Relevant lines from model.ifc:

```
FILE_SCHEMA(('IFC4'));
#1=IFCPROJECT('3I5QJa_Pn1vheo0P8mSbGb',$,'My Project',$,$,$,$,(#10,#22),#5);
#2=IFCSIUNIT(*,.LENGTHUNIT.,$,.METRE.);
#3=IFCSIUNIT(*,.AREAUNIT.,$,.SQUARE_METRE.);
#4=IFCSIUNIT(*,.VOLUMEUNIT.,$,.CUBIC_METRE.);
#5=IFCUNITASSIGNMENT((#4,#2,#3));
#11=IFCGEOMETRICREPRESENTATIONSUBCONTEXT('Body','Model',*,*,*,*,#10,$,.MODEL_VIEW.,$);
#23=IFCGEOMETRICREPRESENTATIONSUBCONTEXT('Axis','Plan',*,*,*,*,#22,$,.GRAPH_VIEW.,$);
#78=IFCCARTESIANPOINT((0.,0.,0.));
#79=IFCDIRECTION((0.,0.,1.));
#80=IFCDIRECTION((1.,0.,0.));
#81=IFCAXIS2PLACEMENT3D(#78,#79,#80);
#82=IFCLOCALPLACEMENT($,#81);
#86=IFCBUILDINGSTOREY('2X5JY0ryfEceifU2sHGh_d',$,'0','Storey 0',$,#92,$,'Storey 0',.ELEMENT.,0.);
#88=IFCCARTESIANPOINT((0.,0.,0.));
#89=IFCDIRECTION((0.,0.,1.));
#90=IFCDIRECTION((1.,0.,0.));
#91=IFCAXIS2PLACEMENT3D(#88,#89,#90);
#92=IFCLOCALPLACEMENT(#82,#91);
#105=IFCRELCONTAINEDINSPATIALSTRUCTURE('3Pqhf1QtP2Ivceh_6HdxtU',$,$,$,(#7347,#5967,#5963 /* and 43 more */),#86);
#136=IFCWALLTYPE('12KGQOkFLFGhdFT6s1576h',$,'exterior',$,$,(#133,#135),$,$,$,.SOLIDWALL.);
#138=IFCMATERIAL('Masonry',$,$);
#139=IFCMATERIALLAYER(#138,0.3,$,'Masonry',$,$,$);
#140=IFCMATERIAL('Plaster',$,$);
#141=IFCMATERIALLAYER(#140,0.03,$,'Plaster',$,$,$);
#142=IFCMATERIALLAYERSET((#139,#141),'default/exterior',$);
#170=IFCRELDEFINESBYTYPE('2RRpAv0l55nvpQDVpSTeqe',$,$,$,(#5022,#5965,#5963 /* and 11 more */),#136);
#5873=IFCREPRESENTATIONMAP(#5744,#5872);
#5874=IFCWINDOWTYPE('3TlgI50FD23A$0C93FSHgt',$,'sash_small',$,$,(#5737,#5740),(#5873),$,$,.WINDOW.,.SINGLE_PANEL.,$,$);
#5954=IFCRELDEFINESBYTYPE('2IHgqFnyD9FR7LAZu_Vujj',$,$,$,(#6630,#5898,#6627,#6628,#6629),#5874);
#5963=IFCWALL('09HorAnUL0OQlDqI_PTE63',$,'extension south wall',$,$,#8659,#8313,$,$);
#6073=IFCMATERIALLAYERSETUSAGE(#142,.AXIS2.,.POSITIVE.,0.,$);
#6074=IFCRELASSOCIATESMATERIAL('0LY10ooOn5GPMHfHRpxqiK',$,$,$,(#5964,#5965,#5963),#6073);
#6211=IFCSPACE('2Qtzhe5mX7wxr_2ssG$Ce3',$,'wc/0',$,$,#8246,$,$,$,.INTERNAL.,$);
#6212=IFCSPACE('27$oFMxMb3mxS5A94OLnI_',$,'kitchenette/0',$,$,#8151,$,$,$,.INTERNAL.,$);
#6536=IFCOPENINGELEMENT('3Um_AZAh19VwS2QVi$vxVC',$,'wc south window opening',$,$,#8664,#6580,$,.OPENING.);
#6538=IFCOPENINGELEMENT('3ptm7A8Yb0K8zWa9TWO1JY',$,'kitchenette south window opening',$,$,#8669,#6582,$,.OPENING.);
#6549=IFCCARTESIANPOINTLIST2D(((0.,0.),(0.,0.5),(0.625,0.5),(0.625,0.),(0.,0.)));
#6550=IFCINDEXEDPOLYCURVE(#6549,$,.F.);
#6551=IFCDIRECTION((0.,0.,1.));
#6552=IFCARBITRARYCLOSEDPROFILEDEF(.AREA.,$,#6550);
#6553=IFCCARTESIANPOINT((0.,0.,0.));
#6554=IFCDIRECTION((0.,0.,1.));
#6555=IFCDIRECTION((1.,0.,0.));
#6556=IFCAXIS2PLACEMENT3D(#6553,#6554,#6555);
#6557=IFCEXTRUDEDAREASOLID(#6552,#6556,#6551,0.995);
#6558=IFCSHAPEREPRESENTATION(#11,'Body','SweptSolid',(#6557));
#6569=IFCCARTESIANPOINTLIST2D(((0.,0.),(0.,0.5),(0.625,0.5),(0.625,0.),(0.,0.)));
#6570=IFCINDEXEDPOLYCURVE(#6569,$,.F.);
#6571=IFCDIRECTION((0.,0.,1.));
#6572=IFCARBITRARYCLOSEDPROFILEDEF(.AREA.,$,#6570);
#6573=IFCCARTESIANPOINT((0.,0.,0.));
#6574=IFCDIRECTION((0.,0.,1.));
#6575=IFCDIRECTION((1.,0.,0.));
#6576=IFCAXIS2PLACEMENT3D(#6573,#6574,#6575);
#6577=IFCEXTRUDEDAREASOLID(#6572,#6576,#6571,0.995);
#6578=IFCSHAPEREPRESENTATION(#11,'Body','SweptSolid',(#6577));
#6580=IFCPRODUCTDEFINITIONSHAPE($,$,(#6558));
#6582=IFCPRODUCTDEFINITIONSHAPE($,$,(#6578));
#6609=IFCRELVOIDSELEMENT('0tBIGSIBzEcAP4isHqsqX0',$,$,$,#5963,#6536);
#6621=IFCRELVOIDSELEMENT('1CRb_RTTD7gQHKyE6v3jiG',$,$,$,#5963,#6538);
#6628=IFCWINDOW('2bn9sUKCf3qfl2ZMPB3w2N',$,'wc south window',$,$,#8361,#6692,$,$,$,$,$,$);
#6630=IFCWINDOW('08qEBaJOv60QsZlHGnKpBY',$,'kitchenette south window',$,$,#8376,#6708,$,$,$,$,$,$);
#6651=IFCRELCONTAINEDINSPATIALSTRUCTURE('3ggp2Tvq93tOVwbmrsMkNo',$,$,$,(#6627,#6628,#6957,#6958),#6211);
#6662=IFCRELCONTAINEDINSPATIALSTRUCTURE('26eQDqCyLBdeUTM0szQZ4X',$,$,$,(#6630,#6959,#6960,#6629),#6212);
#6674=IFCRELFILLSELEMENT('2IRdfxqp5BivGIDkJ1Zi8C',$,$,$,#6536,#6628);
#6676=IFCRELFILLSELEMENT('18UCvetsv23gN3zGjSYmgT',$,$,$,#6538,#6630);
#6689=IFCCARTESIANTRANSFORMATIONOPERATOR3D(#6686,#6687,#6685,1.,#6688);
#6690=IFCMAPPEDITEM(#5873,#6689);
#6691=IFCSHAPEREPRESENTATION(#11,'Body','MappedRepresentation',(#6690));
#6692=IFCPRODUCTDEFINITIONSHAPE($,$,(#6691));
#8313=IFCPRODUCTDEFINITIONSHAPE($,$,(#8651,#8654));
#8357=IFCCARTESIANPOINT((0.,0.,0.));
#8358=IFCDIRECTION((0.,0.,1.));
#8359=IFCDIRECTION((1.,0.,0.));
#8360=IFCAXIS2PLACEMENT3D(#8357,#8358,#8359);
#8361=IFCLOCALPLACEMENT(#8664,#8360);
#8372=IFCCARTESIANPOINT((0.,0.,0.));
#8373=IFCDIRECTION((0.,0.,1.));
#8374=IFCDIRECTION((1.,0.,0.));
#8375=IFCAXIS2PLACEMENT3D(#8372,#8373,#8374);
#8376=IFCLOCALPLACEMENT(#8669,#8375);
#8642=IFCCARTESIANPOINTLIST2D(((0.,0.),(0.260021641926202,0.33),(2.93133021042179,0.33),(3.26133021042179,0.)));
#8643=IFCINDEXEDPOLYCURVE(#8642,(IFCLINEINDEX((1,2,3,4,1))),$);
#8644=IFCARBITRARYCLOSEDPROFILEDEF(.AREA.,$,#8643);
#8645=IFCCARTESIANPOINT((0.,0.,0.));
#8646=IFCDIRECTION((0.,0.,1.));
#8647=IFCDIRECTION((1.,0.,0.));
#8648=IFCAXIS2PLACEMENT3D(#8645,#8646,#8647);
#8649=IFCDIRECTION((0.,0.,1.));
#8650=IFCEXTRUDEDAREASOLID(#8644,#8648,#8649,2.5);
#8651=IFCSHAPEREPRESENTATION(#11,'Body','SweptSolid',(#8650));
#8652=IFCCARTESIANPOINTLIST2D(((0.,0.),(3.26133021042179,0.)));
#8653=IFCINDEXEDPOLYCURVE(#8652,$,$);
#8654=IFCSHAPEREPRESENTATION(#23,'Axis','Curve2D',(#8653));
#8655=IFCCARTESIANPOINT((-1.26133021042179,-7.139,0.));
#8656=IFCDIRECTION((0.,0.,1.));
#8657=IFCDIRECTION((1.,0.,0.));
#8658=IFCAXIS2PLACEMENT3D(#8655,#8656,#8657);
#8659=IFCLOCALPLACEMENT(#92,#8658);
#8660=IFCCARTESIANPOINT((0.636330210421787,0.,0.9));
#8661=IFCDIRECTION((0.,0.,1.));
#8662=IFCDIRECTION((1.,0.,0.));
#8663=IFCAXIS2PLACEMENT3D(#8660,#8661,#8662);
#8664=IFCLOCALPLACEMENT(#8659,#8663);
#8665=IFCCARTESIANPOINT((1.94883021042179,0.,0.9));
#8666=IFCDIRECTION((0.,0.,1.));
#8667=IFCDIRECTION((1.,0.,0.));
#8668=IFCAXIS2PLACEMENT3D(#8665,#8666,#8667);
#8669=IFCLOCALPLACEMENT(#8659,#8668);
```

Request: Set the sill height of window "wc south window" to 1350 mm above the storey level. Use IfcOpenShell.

```python
import numpy as np
import ifcopenshell
import ifcopenshell.api.geometry
import ifcopenshell.geom
import ifcopenshell.util.element
import ifcopenshell.util.placement
import ifcopenshell.util.shape
import ifcopenshell.util.unit

model = ifcopenshell.open("model.ifc")
unit_scale = ifcopenshell.util.unit.calculate_unit_scale(model)

window = model.by_id(6628)
opening = window.FillsVoids[0].RelatingOpeningElement
storey = ifcopenshell.util.element.get_container(window, ifc_class="IfcBuildingStorey")
level = ifcopenshell.util.placement.get_local_placement(storey.ObjectPlacement)[2, 3]

# The opening's origin need not be at the sill, so measure its lowest point.
shape = ifcopenshell.geom.create_shape(ifcopenshell.geom.settings(), opening)
bottom = ifcopenshell.util.shape.get_shape_bottom_elevation(shape, shape.geometry) / unit_scale
dz = level + 1.35 / unit_scale - bottom

shift = np.array([0.0, 0.0, dz])
# The window is placed relative to its opening, so it follows when the opening moves.
matrix = ifcopenshell.util.placement.get_local_placement(opening.ObjectPlacement)
matrix[:3, 3] += shift
ifcopenshell.api.geometry.edit_object_placement(
    model, product=opening, matrix=matrix, is_si=False, should_transform_children=True
)

print(f"moved by {dz * unit_scale:+.3f} m")

model.write("model-out.ifc")
```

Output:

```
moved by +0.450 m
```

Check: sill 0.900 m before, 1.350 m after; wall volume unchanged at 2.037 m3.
